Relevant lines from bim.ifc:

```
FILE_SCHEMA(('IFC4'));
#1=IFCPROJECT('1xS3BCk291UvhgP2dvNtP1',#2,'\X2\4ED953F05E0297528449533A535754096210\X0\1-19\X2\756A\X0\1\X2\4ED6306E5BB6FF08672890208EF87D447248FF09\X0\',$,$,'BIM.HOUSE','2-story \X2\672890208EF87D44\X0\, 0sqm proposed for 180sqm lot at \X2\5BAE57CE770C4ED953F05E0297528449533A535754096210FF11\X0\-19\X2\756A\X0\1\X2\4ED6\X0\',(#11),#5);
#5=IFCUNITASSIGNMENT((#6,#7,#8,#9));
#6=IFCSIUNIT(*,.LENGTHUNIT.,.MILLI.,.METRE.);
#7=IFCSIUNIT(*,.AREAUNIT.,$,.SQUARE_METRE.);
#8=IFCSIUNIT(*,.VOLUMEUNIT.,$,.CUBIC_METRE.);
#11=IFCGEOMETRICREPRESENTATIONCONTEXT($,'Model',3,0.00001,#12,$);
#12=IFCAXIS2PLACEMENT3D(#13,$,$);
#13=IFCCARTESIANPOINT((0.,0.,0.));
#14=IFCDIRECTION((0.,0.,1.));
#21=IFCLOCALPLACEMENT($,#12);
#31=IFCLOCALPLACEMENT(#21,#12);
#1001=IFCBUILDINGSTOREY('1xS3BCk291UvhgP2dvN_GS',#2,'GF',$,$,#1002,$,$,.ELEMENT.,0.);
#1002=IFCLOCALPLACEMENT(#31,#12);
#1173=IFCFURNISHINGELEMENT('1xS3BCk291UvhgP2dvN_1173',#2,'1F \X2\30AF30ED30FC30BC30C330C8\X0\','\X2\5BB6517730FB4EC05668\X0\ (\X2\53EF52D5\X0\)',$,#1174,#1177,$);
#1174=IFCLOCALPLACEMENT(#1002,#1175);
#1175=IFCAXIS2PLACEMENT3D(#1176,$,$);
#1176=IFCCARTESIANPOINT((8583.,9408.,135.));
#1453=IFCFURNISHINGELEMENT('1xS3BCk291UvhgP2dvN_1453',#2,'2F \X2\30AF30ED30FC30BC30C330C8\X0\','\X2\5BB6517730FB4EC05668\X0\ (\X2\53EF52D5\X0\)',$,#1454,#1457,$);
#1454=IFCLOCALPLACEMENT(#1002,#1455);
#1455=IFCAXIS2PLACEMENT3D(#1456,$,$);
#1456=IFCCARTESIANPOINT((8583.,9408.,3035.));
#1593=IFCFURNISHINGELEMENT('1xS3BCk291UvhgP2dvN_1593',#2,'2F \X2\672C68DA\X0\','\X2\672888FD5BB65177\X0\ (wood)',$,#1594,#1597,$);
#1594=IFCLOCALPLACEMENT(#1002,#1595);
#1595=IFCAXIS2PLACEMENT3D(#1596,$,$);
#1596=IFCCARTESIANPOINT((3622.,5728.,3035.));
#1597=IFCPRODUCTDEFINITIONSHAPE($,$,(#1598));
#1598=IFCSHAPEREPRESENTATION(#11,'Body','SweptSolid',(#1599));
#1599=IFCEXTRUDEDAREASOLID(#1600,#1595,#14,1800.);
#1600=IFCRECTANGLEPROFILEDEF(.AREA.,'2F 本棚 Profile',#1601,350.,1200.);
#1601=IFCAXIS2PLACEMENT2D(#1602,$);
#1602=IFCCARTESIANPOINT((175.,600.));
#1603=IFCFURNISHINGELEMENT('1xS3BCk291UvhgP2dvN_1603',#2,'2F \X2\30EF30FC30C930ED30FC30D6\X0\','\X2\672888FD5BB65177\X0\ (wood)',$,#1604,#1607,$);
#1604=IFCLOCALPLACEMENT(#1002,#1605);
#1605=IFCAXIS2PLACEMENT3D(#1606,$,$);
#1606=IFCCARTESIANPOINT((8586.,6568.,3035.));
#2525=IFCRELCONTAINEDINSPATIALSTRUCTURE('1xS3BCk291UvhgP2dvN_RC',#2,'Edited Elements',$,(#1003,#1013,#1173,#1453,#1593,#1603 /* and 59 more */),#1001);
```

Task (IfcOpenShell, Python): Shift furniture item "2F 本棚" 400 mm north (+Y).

```python
import ifcopenshell
import ifcopenshell.api.geometry
import ifcopenshell.util.placement

model = ifcopenshell.open("bim.ifc")

item = model.by_id(1593)
matrix = ifcopenshell.util.placement.get_local_placement(item.ObjectPlacement)
matrix[1, 3] += 400.0
ifcopenshell.api.geometry.edit_object_placement(model, product=item, matrix=matrix, is_si=False)

print(ifcopenshell.util.placement.get_local_placement(item.ObjectPlacement).round(3) + 0.0)

model.write("bim_updated.ifc")
```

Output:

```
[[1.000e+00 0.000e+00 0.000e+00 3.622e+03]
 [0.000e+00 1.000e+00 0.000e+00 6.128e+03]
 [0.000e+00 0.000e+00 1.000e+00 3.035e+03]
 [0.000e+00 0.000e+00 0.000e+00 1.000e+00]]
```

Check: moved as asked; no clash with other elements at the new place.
